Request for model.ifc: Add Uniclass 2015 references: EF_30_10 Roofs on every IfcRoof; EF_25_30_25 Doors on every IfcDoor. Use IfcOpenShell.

First a look at what the model holds.

```python
import ifcopenshell

model = ifcopenshell.open("model.ifc")
print(model.schema)
print("classifications:", [c.Name for c in model.by_type("IfcClassification")])
for ifc_class in ("IfcDoor", "IfcRoof", "IfcStair", "IfcWall", "IfcWindow"):
    print(ifc_class, len(model.by_type(ifc_class)))
```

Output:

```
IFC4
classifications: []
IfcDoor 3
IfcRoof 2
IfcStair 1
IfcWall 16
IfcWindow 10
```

```python
import ifcopenshell
import ifcopenshell.api.classification

model = ifcopenshell.open("model.ifc")

system = ifcopenshell.api.classification.add_classification(model, classification="Uniclass 2015")

codes = {
    "IfcRoof": ("EF_30_10", "Roofs"),
    "IfcDoor": ("EF_25_30_25", "Doors"),
}
for ifc_class, (code, name) in codes.items():
    products = model.by_type(ifc_class)
    ifcopenshell.api.classification.add_reference(
        model, products=products, classification=system, identification=code, name=name
    )
    print(code, len(products))

model.write("model_v2.ifc")
```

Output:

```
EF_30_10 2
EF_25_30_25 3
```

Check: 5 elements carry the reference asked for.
